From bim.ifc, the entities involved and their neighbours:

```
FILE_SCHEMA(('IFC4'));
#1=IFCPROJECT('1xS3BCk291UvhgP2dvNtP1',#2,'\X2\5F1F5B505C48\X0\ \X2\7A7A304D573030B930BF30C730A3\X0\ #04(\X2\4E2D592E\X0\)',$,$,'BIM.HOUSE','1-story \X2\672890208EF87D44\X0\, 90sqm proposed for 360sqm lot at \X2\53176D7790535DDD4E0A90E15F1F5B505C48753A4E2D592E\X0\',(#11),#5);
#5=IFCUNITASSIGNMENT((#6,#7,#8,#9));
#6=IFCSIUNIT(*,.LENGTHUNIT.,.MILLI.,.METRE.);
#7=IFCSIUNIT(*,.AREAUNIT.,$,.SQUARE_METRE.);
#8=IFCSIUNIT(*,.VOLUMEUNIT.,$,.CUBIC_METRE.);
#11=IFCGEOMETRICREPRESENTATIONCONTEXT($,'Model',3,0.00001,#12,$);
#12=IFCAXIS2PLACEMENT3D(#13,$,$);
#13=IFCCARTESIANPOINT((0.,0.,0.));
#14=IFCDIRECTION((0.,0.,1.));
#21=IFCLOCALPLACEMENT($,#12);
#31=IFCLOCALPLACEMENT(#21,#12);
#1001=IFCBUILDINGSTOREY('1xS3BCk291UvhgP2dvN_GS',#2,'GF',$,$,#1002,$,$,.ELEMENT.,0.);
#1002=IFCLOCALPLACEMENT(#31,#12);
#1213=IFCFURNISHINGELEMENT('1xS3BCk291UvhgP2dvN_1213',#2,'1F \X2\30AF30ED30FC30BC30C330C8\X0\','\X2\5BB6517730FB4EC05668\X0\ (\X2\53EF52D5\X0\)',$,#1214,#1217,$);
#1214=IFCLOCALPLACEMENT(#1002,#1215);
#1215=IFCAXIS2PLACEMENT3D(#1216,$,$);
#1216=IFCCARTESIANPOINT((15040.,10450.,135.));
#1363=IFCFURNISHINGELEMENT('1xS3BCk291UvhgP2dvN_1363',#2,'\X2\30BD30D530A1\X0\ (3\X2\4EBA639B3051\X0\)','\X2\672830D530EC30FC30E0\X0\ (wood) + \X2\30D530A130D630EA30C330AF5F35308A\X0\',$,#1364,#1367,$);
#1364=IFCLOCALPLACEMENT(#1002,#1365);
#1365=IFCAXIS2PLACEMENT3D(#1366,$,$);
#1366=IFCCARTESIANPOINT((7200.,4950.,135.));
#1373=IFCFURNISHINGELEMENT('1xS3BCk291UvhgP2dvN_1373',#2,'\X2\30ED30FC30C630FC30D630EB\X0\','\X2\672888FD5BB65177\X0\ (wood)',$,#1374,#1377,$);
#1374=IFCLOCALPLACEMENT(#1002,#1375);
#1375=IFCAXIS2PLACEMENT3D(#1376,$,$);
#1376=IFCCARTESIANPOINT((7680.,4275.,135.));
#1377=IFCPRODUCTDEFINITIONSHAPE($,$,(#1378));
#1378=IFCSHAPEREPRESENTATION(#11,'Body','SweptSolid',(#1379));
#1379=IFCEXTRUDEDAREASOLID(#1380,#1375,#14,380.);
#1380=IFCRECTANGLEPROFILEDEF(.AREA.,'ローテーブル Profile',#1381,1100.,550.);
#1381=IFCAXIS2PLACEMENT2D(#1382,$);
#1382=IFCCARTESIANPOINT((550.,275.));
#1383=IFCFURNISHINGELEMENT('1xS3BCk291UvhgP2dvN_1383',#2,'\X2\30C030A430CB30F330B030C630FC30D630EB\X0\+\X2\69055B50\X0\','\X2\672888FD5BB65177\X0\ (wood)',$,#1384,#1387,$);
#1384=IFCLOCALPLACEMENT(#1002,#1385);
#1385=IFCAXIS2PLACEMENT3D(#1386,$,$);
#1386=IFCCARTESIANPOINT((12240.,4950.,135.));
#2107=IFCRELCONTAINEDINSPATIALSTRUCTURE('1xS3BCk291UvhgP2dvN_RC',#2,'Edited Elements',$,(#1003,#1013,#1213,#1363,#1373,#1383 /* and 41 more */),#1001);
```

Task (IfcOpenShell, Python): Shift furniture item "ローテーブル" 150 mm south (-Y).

```python
import ifcopenshell
import ifcopenshell.api.geometry
import ifcopenshell.util.placement

model = ifcopenshell.open("bim.ifc")

item = model.by_id(1373)
matrix = ifcopenshell.util.placement.get_local_placement(item.ObjectPlacement)
matrix[1, 3] -= 150.0
ifcopenshell.api.geometry.edit_object_placement(model, product=item, matrix=matrix, is_si=False)

print(ifcopenshell.util.placement.get_local_placement(item.ObjectPlacement).round(3) + 0.0)

model.write("bim_edited.ifc")
```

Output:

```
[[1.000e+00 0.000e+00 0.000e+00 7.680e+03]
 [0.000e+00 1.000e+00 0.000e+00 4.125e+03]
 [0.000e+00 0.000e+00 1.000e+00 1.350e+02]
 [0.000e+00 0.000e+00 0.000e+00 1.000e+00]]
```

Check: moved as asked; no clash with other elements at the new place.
